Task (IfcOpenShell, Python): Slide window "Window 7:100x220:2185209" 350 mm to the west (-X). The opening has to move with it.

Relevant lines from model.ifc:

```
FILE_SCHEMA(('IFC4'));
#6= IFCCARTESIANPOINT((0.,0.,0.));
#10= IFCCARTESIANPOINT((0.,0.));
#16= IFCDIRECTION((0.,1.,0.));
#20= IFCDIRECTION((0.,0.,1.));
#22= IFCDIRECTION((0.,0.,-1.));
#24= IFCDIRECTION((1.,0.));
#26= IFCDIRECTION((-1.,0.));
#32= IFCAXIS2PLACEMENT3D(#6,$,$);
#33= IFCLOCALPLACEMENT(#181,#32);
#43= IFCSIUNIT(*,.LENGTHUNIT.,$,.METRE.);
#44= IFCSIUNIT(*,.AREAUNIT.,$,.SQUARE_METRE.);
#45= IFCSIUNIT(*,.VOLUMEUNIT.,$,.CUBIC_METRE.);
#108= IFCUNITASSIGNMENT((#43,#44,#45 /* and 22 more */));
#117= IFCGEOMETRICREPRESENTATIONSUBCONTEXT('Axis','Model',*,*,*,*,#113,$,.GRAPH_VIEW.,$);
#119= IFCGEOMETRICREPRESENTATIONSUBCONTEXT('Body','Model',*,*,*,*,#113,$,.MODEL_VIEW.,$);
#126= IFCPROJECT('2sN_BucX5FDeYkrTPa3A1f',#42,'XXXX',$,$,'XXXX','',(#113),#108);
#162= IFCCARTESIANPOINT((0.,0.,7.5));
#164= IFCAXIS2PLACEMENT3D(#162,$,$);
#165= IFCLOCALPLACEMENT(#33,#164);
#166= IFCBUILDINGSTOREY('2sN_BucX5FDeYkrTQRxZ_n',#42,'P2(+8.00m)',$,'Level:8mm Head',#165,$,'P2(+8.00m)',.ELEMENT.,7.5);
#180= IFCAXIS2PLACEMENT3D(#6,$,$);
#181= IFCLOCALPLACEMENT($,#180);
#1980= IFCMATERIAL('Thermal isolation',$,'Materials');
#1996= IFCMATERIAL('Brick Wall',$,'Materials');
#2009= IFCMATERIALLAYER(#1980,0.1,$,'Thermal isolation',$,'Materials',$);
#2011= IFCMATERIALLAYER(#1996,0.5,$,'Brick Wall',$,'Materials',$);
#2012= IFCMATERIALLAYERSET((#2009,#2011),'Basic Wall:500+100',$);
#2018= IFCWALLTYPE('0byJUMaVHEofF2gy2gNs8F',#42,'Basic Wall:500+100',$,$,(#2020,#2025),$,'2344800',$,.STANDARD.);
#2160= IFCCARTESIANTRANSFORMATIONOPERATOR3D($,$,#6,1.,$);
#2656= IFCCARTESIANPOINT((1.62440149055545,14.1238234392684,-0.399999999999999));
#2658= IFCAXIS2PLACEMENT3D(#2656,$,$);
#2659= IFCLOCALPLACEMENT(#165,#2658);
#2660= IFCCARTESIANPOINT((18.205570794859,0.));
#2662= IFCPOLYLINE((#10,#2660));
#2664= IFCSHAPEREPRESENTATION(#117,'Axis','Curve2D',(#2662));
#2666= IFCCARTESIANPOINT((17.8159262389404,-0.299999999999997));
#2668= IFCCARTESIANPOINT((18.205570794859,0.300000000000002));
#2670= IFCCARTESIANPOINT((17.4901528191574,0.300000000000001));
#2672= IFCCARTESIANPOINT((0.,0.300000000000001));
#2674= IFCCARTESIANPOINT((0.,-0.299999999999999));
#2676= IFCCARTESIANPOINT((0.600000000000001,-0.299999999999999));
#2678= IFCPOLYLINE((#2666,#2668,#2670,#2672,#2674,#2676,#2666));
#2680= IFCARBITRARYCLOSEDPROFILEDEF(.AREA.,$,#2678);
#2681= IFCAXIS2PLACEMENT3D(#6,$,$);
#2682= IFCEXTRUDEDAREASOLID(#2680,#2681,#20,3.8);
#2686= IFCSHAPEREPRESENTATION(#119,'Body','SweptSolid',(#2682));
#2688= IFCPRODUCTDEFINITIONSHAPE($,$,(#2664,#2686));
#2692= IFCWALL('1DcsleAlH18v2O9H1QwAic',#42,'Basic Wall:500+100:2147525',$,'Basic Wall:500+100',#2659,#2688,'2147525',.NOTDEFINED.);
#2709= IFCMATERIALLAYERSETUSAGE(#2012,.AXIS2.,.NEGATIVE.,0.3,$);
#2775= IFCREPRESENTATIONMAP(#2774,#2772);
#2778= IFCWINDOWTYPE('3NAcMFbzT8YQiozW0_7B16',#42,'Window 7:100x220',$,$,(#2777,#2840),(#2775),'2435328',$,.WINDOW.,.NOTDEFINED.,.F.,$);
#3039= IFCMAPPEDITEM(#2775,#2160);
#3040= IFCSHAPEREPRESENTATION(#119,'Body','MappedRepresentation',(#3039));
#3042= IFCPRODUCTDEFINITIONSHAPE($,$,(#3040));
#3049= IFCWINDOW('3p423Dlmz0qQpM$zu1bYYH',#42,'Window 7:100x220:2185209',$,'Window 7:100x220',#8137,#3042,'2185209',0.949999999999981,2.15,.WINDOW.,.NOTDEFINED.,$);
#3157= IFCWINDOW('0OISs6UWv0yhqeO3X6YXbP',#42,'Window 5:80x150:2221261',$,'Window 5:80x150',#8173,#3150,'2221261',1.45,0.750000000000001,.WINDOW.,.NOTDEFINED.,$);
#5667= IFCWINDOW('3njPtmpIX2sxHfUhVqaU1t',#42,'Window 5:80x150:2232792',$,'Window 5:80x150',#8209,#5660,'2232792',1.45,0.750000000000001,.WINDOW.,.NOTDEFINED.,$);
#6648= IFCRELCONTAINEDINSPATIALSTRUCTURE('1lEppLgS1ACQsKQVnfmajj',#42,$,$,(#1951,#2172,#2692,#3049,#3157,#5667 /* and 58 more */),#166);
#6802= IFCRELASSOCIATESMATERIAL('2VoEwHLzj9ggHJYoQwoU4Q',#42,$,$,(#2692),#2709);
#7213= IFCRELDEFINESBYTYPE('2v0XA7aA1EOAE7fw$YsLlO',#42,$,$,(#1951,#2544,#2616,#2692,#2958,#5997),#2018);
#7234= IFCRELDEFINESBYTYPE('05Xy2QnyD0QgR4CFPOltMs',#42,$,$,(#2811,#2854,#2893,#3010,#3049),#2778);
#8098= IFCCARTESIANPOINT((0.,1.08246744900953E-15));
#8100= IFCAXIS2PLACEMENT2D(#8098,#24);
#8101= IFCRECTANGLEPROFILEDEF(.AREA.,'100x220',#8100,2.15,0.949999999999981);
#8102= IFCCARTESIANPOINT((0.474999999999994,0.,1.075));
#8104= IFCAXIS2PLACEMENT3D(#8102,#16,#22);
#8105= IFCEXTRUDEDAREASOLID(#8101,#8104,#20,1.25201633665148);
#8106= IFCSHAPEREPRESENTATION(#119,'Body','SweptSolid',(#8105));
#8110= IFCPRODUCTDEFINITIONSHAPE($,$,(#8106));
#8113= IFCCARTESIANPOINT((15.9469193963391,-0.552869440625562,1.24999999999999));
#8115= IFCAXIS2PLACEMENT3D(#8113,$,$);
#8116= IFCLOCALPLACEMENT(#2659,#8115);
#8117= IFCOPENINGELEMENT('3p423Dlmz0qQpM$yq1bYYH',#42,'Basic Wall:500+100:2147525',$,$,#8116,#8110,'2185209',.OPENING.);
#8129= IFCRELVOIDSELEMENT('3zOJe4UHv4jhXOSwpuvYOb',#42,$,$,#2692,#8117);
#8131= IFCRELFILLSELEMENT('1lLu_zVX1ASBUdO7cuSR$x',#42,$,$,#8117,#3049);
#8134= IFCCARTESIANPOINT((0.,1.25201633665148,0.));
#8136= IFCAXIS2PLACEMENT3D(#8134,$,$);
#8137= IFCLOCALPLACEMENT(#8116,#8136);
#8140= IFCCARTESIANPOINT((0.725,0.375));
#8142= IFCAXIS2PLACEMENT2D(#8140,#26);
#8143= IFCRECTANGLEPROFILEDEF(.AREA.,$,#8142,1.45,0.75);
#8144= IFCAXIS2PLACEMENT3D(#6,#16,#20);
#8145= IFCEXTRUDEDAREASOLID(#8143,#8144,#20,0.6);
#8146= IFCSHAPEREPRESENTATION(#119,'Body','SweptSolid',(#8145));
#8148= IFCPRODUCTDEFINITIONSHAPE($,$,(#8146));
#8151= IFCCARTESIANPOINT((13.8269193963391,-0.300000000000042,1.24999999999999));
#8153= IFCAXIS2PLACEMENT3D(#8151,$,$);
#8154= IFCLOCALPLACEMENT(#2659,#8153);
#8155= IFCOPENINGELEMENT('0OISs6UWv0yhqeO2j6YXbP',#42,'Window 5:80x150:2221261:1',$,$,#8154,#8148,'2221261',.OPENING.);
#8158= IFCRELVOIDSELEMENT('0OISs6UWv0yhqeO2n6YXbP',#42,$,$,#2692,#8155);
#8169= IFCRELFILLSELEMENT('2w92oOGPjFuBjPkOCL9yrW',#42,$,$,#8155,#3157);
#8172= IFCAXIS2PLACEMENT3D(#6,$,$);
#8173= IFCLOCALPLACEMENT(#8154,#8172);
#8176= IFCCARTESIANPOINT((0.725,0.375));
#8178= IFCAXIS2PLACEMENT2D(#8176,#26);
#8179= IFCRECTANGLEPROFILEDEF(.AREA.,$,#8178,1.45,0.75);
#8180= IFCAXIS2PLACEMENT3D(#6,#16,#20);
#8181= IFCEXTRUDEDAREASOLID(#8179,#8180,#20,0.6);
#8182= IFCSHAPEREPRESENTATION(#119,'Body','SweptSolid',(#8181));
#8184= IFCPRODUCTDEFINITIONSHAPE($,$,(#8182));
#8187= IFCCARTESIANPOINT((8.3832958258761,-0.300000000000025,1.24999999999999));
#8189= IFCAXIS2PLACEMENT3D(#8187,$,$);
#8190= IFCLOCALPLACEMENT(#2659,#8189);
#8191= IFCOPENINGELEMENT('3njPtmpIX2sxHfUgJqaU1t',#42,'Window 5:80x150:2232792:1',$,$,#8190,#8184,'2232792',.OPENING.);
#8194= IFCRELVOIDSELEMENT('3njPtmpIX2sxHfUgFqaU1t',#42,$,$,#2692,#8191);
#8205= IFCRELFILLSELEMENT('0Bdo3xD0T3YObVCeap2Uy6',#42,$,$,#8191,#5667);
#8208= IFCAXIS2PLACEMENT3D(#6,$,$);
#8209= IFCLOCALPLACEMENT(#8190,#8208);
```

```python
import ifcopenshell
import ifcopenshell.api.geometry
import ifcopenshell.util.placement
import ifcopenshell.util.unit

model = ifcopenshell.open("model.ifc")
unit_scale = ifcopenshell.util.unit.calculate_unit_scale(model)

window = model.by_id(3049)
opening = window.FillsVoids[0].RelatingOpeningElement
wall = opening.VoidsElements[0].RelatingBuildingElement

wall_matrix = ifcopenshell.util.placement.get_local_placement(wall.ObjectPlacement)
shift = wall_matrix[:3, 0] * -0.35 / unit_scale
before = ifcopenshell.util.placement.get_local_placement(window.ObjectPlacement)[:3, 3].copy()

# The window is placed relative to its opening, so it follows when the opening moves.
matrix = ifcopenshell.util.placement.get_local_placement(opening.ObjectPlacement)
matrix[:3, 3] += shift
ifcopenshell.api.geometry.edit_object_placement(
    model, product=opening, matrix=matrix, is_si=False, should_transform_children=True
)

after = ifcopenshell.util.placement.get_local_placement(window.ObjectPlacement)[:3, 3]
print("window moved by", (after - before).round(3) + 0.0)

model.write("model_edited.ifc")
```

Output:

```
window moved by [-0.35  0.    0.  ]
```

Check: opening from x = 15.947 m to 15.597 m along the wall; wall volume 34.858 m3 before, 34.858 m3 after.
